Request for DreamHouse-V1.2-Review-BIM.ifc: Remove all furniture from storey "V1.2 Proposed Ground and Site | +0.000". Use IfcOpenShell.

First a look at what the model holds.

```python
import ifcopenshell
import ifcopenshell.util.element

model = ifcopenshell.open("DreamHouse-V1.2-Review-BIM.ifc")
print(model.schema)
storey = next(s for s in model.by_type("IfcBuildingStorey") if s.Name == "V1.2 Proposed Ground and Site | +0.000")
furniture = [e for e in ifcopenshell.util.element.get_decomposition(storey) if e.is_a("IfcFurnishingElement")]
seen = {}
for e in furniture:
    element_type = ifcopenshell.util.element.get_type(e)
    name = element_type.Name if element_type not in (None, e) else None
    seen[name] = seen.get(name, 0) + 1
for name, count in sorted(seen.items(), key=str):
    print(count, "x", name)
```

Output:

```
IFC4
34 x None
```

```python
import ifcopenshell
import ifcopenshell.api.root
import ifcopenshell.util.element

model = ifcopenshell.open("DreamHouse-V1.2-Review-BIM.ifc")

storey = next(s for s in model.by_type("IfcBuildingStorey") if s.Name == "V1.2 Proposed Ground and Site | +0.000")
furniture = [e for e in ifcopenshell.util.element.get_decomposition(storey) if e.is_a("IfcFurnishingElement")]

for e in furniture:
    ifcopenshell.api.root.remove_product(model, product=e)
print(len(furniture), "removed")

model.write("DreamHouse-V1.2-Review-BIM_v2.ifc")
```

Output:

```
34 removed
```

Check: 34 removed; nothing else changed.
